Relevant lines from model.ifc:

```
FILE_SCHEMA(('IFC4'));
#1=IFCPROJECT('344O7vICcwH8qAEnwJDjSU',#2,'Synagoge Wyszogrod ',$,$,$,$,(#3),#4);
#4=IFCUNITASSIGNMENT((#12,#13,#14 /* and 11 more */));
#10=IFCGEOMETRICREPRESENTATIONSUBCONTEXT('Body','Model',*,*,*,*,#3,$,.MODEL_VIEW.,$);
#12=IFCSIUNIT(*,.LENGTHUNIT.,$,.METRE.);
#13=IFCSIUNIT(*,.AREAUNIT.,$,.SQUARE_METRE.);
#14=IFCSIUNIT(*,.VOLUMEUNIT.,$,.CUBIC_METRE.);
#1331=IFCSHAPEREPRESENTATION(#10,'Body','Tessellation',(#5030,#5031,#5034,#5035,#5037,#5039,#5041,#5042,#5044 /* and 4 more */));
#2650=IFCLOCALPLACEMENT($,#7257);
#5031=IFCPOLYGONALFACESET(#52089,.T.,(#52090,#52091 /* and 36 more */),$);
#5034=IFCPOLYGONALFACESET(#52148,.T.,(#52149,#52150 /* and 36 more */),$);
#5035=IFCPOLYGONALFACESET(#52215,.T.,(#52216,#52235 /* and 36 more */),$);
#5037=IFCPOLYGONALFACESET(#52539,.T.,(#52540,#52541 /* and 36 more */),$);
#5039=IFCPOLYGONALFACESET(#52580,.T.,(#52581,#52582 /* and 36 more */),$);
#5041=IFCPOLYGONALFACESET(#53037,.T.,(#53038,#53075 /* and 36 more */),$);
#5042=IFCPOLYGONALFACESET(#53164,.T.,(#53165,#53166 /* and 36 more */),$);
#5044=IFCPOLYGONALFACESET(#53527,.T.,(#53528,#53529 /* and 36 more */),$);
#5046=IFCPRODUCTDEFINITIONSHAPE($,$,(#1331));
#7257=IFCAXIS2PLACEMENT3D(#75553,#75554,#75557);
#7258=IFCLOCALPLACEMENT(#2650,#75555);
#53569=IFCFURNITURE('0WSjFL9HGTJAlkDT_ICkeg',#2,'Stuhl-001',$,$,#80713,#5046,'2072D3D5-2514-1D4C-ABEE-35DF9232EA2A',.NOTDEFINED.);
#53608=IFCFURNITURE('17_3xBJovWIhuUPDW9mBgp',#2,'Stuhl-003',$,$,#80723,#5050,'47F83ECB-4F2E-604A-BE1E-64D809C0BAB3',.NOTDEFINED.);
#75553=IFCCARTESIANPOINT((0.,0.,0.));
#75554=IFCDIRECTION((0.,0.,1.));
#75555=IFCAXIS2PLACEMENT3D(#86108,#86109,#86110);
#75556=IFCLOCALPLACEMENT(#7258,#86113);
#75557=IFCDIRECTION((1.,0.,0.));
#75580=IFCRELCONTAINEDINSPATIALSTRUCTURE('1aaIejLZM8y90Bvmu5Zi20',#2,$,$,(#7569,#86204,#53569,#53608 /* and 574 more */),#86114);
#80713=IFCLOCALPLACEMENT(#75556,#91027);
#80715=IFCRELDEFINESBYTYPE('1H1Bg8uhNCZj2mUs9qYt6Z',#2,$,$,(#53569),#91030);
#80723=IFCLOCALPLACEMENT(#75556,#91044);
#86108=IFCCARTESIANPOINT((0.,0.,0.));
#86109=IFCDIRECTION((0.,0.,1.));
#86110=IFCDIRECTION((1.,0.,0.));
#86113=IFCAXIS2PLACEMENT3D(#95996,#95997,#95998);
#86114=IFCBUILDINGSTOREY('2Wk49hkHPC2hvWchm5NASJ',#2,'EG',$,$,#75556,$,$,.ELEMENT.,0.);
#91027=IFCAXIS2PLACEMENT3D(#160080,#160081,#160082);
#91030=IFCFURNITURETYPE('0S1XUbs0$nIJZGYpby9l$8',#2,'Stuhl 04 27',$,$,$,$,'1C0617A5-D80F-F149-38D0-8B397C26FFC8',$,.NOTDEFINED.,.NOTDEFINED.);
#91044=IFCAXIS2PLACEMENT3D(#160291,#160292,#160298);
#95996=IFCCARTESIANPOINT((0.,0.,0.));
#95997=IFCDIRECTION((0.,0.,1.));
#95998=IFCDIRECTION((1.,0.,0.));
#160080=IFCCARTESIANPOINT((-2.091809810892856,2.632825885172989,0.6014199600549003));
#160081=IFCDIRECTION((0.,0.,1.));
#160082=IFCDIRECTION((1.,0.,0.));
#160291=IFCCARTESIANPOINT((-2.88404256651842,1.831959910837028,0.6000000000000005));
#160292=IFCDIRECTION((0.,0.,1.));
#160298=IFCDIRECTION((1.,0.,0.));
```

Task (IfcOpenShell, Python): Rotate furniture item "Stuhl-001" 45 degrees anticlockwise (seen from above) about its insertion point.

```python
import ifcopenshell
import ifcopenshell.api.geometry
import ifcopenshell.util.placement

model = ifcopenshell.open("model.ifc")

item = model.by_id(53569)
matrix = ifcopenshell.util.placement.get_local_placement(item.ObjectPlacement)
matrix = matrix @ ifcopenshell.util.placement.rotation(45, "Z")
ifcopenshell.api.geometry.edit_object_placement(model, product=item, matrix=matrix, is_si=False)

print(ifcopenshell.util.placement.get_local_placement(item.ObjectPlacement).round(3) + 0.0)

model.write("model_updated.ifc")
```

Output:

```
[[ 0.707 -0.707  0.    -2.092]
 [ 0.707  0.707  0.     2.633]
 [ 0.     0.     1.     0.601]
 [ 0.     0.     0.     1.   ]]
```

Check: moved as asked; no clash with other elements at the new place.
